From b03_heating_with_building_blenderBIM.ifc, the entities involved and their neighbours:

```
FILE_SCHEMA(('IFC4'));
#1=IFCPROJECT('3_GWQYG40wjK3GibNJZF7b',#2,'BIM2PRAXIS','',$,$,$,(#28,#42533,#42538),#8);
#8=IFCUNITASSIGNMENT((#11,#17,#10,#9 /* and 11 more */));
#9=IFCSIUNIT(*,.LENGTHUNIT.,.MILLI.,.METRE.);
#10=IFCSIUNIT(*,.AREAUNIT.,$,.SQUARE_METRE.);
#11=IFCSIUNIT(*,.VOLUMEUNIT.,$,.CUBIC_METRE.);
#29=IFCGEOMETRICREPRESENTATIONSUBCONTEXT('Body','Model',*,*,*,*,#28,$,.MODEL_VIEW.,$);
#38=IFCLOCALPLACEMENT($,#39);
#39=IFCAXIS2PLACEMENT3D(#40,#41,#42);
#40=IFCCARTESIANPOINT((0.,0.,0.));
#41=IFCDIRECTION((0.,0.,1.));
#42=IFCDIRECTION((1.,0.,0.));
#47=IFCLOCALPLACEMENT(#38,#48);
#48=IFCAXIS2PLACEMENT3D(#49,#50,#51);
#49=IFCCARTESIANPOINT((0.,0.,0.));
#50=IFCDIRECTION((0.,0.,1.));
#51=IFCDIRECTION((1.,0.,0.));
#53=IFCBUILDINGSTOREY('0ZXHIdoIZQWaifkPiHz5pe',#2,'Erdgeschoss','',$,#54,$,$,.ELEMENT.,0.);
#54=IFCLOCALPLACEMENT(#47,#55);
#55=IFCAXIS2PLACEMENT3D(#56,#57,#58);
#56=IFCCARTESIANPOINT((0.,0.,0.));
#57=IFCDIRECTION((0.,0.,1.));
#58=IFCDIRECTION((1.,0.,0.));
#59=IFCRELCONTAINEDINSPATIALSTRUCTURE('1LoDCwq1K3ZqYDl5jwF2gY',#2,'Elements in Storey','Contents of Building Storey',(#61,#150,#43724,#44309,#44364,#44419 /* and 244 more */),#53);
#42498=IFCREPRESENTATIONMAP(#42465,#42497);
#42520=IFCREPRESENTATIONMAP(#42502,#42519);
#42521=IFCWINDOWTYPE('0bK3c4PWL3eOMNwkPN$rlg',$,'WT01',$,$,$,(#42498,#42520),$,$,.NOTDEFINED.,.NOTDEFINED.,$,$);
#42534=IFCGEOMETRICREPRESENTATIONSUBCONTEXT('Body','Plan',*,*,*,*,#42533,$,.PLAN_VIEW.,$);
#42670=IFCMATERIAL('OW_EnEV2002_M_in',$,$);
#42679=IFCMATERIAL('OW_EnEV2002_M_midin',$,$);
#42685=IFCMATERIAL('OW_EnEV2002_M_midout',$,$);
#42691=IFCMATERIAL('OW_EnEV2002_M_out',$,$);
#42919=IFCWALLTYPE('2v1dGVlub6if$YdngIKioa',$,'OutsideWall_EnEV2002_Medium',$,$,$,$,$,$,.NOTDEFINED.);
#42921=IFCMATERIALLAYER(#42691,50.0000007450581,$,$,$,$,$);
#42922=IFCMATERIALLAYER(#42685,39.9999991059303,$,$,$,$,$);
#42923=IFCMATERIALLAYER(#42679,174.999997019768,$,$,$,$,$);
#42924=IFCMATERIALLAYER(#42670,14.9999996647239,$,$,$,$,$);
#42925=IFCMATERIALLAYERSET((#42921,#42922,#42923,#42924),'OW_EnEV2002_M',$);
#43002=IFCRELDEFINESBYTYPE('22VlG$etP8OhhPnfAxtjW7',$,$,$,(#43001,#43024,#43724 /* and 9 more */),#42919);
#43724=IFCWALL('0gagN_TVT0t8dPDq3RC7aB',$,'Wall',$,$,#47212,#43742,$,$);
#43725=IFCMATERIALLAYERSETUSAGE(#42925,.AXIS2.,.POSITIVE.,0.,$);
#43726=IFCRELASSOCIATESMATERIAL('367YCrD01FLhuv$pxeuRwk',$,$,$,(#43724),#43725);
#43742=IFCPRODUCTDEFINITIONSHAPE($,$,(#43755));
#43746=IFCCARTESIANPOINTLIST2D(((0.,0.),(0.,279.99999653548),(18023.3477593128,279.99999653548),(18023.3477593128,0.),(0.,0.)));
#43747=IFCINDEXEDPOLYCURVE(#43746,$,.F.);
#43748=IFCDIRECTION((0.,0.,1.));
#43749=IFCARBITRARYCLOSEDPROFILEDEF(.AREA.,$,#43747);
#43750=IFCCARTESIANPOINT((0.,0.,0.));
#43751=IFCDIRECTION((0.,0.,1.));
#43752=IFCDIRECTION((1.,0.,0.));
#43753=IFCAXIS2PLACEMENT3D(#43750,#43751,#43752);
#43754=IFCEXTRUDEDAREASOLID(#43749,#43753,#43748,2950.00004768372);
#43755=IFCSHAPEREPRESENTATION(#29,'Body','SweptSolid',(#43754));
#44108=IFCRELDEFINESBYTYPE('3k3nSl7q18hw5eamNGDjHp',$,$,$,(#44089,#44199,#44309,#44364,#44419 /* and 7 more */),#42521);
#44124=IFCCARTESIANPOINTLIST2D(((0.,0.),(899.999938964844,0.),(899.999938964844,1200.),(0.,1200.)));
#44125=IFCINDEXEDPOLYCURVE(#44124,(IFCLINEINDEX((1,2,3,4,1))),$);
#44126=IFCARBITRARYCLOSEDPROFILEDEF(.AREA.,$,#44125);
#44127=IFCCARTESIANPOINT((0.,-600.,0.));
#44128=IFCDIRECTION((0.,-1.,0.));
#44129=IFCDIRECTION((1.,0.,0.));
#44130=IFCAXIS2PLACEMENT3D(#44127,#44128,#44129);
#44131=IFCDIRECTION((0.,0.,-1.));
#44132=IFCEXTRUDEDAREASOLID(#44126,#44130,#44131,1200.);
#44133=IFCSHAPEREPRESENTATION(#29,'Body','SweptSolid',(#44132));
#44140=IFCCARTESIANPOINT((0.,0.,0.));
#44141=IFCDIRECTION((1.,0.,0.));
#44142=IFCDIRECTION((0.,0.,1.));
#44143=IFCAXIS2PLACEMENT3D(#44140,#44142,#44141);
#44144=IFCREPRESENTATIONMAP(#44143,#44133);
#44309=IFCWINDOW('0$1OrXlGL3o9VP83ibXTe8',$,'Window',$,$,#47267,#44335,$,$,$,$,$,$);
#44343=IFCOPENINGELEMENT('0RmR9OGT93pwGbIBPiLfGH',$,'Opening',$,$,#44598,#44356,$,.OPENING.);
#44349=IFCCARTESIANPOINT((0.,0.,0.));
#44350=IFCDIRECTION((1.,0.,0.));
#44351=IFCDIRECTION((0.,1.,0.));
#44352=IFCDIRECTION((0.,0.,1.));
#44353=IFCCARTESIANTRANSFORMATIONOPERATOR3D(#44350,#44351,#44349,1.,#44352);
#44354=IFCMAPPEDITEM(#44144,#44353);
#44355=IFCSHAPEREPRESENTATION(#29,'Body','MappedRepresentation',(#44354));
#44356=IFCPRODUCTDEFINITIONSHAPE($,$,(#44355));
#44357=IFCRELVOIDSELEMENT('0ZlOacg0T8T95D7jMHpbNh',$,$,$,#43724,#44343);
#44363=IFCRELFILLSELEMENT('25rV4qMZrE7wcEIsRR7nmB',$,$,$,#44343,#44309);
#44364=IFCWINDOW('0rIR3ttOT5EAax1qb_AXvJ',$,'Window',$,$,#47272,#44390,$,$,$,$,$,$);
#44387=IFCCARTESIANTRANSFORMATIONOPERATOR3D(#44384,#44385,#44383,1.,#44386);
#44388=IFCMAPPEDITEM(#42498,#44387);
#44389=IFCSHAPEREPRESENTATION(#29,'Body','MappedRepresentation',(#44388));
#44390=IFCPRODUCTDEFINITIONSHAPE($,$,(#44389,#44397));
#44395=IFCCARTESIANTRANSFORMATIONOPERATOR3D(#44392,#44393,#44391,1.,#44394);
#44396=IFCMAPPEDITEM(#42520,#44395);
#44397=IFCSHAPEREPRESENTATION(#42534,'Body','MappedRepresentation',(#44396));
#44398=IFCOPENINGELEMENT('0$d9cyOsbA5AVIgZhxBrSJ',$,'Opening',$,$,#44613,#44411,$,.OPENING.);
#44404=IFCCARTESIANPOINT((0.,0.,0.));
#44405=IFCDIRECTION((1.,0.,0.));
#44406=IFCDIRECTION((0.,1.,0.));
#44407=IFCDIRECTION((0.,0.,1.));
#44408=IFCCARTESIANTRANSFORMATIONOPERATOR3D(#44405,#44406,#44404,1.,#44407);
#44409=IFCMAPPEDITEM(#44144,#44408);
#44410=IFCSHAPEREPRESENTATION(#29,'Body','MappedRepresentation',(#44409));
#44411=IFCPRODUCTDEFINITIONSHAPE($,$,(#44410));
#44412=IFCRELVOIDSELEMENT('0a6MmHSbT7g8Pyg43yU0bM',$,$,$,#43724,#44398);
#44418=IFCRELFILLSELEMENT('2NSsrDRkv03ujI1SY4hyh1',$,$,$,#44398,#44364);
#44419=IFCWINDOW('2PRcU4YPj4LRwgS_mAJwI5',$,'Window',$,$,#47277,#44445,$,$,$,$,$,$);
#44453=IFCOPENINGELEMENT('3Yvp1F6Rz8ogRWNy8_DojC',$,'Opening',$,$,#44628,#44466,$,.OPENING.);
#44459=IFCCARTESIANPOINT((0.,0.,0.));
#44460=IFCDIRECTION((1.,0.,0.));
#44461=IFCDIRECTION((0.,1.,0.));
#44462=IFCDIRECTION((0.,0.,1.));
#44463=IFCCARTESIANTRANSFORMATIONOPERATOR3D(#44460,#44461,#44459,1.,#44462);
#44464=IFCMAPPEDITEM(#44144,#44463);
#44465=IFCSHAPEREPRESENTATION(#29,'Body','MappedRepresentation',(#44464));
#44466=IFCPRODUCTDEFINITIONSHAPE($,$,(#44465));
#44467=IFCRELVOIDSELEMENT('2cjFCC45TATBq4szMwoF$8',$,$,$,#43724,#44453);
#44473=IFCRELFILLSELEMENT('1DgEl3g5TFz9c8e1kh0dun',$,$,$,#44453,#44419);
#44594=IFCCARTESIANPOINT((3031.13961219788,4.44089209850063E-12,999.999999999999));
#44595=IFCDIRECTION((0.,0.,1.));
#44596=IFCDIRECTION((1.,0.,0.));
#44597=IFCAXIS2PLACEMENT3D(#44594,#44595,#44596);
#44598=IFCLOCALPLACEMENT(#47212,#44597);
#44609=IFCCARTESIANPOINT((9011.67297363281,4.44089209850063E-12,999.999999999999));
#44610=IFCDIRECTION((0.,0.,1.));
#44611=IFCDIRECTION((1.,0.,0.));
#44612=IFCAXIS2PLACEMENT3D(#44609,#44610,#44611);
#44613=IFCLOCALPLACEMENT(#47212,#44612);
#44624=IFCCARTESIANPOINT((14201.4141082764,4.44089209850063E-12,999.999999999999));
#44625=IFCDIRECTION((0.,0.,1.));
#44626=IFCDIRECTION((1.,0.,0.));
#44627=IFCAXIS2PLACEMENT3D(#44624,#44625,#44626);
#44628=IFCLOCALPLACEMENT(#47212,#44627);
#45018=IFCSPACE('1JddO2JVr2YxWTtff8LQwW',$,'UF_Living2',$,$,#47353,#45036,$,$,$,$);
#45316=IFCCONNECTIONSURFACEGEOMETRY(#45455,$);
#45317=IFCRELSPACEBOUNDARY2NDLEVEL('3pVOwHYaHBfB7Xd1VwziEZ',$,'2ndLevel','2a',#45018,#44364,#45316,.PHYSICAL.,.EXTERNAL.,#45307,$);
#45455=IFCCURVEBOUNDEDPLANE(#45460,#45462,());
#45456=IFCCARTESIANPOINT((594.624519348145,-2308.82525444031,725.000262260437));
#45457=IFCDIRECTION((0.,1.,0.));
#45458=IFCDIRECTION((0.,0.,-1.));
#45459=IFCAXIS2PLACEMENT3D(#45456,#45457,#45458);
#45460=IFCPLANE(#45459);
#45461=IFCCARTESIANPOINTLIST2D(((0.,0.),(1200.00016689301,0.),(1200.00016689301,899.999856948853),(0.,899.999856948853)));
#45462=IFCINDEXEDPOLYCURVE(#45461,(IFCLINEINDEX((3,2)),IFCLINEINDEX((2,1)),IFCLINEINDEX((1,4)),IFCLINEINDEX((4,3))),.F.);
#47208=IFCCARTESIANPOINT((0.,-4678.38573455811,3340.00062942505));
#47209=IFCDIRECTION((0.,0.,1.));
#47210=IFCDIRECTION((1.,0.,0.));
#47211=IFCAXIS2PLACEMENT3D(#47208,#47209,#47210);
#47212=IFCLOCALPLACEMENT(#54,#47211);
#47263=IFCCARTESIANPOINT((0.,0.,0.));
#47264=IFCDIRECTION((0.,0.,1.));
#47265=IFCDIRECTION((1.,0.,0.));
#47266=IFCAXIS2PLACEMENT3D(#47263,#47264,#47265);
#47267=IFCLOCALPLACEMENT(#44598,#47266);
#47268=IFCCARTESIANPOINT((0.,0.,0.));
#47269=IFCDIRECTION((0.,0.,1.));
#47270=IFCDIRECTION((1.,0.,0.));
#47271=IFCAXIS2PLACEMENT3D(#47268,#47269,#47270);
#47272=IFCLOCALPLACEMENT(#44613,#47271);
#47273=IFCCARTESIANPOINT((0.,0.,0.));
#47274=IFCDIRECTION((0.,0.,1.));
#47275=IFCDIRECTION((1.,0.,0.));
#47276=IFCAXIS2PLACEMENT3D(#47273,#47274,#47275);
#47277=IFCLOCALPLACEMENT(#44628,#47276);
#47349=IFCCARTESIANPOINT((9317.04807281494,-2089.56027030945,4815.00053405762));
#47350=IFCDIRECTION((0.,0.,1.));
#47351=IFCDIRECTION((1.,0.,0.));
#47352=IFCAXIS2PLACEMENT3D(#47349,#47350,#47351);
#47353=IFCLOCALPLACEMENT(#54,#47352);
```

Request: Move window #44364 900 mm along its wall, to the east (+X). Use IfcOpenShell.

```python
import numpy as np
import ifcopenshell
import ifcopenshell.api.geometry
import ifcopenshell.util.placement
import ifcopenshell.util.unit

model = ifcopenshell.open("b03_heating_with_building_blenderBIM.ifc")
unit_scale = ifcopenshell.util.unit.calculate_unit_scale(model)

window = model.by_id(44364)
opening = window.FillsVoids[0].RelatingOpeningElement
wall = opening.VoidsElements[0].RelatingBuildingElement

wall_matrix = ifcopenshell.util.placement.get_local_placement(wall.ObjectPlacement)
shift = wall_matrix[:3, 0] * 0.9 / unit_scale
before = ifcopenshell.util.placement.get_local_placement(window.ObjectPlacement)[:3, 3].copy()

# The window is placed relative to its opening, so it follows when the opening moves.
matrix = ifcopenshell.util.placement.get_local_placement(opening.ObjectPlacement)
matrix[:3, 3] += shift
ifcopenshell.api.geometry.edit_object_placement(
    model, product=opening, matrix=matrix, is_si=False, should_transform_children=True
)

# Space boundary surfaces are stored in each space's coordinates; move them too.
for rel in window.ProvidesBoundaries:
    if not rel.ConnectionGeometry:
        continue
    surface = rel.ConnectionGeometry.SurfaceOnRelatingElement.BasisSurface
    space_matrix = ifcopenshell.util.placement.get_local_placement(rel.RelatingSpace.ObjectPlacement)
    point = np.array(surface.Position.Location.Coordinates) + space_matrix[:3, :3].T @ shift
    surface.Position = model.createIfcAxis2Placement3D(
        model.createIfcCartesianPoint(point.tolist()), surface.Position.Axis, surface.Position.RefDirection
    )

after = ifcopenshell.util.placement.get_local_placement(window.ObjectPlacement)[:3, 3]
print("window moved by", (after - before).round(3) + 0.0)

model.write("b03_heating_with_building_blenderBIM-out.ifc")
```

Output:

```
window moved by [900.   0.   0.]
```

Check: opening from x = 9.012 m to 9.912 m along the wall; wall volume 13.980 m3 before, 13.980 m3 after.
